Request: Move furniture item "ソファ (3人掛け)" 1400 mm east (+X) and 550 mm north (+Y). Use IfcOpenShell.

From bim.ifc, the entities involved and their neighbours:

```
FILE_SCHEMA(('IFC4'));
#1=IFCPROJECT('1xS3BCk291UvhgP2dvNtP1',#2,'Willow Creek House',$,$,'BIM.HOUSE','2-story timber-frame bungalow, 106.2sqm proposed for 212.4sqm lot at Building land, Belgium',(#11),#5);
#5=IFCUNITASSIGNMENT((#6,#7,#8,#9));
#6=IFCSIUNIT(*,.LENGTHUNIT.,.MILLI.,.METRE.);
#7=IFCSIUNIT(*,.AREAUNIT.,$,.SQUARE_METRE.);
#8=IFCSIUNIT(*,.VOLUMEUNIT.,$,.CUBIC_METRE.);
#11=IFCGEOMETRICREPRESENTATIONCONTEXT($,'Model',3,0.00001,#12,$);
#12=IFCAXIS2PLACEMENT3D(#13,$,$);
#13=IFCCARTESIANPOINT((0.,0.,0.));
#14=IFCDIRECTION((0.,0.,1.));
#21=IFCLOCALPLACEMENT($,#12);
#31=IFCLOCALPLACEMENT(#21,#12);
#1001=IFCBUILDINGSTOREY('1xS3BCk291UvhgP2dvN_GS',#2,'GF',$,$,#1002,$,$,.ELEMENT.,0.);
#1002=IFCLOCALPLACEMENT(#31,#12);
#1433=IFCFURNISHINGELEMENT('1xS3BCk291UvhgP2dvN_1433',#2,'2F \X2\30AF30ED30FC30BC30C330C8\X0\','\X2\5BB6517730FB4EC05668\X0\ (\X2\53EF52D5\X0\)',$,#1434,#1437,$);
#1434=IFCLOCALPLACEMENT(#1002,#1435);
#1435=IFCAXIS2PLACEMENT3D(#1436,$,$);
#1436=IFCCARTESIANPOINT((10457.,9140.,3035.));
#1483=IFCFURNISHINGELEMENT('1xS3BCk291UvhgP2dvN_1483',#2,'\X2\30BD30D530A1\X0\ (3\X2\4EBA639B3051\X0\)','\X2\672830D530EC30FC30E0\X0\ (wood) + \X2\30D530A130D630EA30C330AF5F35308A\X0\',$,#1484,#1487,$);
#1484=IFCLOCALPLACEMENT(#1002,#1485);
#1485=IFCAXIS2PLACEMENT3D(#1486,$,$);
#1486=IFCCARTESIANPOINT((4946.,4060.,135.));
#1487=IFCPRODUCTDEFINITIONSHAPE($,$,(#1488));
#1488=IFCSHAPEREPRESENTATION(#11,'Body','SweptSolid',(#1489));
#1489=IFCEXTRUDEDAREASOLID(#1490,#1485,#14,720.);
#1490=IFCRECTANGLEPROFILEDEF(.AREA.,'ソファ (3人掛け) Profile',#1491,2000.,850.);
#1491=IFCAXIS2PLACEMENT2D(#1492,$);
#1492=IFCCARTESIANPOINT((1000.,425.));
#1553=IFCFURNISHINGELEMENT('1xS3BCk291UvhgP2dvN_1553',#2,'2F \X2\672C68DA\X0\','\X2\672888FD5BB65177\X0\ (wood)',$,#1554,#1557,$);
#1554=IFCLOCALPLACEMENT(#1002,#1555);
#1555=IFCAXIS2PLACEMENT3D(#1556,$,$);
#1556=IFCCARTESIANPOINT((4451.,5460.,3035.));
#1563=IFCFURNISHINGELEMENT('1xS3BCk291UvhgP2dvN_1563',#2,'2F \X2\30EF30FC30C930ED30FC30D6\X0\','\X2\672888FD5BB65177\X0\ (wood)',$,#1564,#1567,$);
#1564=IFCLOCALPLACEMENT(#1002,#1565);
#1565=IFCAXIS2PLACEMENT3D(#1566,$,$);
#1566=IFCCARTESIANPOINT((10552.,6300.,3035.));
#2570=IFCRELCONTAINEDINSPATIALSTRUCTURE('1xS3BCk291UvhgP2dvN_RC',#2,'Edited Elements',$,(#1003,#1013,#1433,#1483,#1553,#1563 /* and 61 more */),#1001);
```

```python
import ifcopenshell
import ifcopenshell.api.geometry
import ifcopenshell.util.placement

model = ifcopenshell.open("bim.ifc")

item = model.by_guid("1xS3BCk291UvhgP2dvN_1483")
matrix = ifcopenshell.util.placement.get_local_placement(item.ObjectPlacement)
matrix[0, 3] += 1400.0
matrix[1, 3] += 550.0
ifcopenshell.api.geometry.edit_object_placement(model, product=item, matrix=matrix, is_si=False)

print(ifcopenshell.util.placement.get_local_placement(item.ObjectPlacement).round(3) + 0.0)

model.write("bim_updated.ifc")
```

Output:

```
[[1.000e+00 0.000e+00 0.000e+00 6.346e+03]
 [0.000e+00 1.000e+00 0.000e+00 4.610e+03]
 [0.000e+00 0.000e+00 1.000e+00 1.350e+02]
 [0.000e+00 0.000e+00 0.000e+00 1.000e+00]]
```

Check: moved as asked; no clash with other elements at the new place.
